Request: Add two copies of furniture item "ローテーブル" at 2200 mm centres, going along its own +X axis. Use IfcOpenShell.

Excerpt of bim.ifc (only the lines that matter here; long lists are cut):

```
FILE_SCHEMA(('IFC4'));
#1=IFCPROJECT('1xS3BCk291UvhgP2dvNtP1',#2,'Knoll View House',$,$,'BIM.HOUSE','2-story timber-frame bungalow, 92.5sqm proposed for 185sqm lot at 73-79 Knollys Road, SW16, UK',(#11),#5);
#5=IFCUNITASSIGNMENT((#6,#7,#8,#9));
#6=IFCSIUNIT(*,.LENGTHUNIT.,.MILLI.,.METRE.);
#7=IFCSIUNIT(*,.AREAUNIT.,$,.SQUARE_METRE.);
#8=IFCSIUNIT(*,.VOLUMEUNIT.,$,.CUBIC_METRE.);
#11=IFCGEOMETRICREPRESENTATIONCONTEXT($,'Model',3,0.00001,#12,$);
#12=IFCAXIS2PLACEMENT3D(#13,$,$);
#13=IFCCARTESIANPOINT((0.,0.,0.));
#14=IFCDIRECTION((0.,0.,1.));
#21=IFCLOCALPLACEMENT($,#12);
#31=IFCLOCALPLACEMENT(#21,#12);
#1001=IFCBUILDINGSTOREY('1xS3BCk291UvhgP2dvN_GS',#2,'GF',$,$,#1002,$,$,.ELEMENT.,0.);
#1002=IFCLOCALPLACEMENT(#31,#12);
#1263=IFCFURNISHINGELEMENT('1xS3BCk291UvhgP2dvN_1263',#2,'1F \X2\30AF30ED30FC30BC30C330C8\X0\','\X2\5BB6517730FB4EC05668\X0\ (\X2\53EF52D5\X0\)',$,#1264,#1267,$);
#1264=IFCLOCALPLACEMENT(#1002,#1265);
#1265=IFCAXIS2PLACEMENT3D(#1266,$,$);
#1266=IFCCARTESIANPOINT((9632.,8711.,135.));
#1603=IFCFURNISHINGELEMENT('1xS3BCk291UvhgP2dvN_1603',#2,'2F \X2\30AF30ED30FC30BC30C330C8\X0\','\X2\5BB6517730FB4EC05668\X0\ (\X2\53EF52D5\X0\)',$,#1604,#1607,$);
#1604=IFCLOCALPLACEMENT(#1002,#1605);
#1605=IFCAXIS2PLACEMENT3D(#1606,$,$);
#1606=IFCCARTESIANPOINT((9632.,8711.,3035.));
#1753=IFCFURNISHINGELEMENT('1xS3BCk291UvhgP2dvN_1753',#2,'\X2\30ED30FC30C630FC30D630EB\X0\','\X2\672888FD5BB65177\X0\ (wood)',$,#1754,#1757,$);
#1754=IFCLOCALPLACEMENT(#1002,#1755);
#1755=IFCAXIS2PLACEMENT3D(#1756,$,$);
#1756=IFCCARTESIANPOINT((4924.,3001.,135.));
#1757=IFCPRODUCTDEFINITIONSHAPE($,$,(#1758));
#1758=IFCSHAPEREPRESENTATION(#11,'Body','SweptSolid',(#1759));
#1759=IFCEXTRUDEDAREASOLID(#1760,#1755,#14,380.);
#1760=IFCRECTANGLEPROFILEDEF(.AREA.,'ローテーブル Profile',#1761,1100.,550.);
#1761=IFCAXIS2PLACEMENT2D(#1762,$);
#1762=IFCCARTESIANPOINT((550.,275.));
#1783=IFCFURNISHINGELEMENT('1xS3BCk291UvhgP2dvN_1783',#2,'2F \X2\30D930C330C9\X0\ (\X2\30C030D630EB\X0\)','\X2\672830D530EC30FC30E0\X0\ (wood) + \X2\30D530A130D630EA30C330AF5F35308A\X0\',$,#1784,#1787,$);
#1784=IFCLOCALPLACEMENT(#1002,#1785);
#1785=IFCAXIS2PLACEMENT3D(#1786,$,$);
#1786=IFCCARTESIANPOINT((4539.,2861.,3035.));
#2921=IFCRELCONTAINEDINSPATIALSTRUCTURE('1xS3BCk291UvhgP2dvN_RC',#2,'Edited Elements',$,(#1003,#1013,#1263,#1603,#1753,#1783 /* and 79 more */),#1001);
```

```python
import ifcopenshell
import ifcopenshell.api.geometry
import ifcopenshell.api.root
import ifcopenshell.util.element
import ifcopenshell.util.placement
import ifcopenshell.util.unit

model = ifcopenshell.open("bim.ifc")
unit_scale = ifcopenshell.util.unit.calculate_unit_scale(model)


def reuse_history(source, copy):
    """copy_class also copies each property set's owner history, people and application; keep the originals."""
    for rel in copy.IsDefinedBy:
        if rel.is_a("IfcRelDefinesByProperties") and (history := rel.RelatingPropertyDefinition.OwnerHistory):
            rel.RelatingPropertyDefinition.OwnerHistory = source.OwnerHistory
            ifcopenshell.util.element.remove_deep2(model, history)


source = model.by_guid("1xS3BCk291UvhgP2dvN_1753")
base = ifcopenshell.util.placement.get_local_placement(source.ObjectPlacement)
step = base[:3, 0] * 2.2 / unit_scale

for i in range(1, 3):
    copy = ifcopenshell.api.root.copy_class(model, product=source)
    copy.Representation = ifcopenshell.util.element.copy_deep(
        model, source.Representation, exclude=["IfcGeometricRepresentationContext", "IfcRepresentationMap"]
    )
    reuse_history(source, copy)
    matrix = base.copy()
    matrix[:3, 3] += i * step
    print("added at", matrix[:3, 3].round(3) + 0.0)
    ifcopenshell.api.geometry.edit_object_placement(model, product=copy, matrix=matrix, is_si=False)

model.write("bim_edited.ifc")
```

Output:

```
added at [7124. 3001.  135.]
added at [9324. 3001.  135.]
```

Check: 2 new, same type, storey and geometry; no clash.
